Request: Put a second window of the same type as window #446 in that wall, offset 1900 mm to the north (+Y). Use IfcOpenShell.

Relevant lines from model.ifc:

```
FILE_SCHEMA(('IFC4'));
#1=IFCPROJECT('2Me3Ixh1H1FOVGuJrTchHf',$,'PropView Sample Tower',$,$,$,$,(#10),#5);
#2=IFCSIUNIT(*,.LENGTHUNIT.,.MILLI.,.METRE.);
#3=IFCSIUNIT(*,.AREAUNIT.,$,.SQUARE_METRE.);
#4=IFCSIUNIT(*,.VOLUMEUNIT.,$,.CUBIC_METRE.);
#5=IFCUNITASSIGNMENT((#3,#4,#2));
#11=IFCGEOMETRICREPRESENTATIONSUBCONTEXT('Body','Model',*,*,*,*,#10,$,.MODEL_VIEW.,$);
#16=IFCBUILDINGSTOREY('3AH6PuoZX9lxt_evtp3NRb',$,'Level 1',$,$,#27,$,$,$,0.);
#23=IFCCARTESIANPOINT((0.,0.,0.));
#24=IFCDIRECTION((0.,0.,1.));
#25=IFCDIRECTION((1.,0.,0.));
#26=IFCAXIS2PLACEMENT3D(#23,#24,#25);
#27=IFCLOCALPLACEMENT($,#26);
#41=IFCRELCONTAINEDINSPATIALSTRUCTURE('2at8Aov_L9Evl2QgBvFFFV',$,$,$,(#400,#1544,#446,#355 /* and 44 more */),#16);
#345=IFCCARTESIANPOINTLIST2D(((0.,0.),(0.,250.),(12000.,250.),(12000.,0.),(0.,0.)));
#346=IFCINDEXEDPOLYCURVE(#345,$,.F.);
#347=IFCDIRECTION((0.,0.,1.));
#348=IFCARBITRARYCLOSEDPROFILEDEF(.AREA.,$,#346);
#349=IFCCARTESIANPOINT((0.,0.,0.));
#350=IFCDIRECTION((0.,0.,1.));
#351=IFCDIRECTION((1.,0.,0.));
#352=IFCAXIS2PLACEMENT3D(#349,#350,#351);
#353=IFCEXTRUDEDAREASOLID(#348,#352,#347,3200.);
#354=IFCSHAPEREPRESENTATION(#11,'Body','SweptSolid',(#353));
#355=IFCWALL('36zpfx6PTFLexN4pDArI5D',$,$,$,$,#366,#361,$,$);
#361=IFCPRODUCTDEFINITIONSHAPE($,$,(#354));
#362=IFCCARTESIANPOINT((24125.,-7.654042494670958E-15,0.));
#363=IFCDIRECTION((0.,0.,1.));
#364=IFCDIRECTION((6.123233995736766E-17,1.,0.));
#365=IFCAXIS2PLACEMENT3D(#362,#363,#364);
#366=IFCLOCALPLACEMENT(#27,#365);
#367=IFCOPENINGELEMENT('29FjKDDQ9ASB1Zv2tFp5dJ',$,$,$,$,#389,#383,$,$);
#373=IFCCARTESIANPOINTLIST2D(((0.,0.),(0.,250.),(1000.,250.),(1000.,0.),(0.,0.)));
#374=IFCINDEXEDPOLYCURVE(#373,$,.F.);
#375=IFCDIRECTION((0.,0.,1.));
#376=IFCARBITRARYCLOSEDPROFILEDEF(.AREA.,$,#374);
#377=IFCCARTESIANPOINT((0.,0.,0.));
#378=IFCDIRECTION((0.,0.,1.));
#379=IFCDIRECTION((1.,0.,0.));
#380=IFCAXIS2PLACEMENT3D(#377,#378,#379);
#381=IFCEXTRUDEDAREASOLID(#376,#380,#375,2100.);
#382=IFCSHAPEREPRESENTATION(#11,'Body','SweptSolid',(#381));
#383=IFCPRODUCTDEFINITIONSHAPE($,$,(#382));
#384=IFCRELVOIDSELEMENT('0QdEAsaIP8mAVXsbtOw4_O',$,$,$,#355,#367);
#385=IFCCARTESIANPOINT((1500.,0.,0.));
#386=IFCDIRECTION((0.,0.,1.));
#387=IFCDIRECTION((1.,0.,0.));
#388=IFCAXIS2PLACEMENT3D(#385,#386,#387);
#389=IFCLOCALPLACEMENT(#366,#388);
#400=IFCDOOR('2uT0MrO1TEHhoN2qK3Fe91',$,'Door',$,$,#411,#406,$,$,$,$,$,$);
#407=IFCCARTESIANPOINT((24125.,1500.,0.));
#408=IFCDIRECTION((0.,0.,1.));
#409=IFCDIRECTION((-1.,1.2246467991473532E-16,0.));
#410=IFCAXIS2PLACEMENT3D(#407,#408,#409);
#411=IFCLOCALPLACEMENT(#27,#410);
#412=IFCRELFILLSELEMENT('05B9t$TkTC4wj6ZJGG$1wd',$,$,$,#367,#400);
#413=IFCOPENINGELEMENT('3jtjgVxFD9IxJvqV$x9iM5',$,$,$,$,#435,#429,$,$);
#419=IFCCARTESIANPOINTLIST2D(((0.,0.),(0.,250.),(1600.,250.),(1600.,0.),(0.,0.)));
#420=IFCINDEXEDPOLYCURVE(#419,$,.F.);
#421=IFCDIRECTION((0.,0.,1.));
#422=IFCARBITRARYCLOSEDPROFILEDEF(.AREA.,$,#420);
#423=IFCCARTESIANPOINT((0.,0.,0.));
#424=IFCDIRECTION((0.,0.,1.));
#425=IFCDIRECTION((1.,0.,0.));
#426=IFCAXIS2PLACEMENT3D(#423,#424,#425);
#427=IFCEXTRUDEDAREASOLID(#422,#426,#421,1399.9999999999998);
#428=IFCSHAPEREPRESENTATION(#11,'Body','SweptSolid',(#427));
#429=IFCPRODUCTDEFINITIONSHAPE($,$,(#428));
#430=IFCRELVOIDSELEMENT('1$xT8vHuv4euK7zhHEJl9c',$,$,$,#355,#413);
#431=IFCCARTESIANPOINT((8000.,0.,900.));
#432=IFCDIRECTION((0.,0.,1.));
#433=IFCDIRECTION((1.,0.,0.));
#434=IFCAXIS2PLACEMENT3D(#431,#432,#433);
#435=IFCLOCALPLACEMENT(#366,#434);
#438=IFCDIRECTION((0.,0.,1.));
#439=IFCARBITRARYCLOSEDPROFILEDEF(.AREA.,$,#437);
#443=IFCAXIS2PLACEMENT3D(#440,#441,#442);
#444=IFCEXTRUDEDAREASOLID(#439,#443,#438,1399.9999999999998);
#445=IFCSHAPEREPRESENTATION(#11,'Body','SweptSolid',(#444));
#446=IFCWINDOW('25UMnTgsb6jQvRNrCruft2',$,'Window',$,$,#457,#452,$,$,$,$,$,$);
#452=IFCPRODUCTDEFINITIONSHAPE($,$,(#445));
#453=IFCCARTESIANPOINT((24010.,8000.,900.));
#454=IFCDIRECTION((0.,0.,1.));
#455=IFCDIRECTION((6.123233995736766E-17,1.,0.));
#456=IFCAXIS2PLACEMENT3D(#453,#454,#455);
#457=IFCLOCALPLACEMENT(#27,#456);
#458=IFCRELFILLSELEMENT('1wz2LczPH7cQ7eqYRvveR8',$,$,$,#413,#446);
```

```python
import ifcopenshell
import ifcopenshell.api.feature
import ifcopenshell.api.geometry
import ifcopenshell.api.root
import ifcopenshell.geom
import ifcopenshell.util.element
import ifcopenshell.util.placement
import ifcopenshell.util.shape
import ifcopenshell.util.unit

model = ifcopenshell.open("model.ifc")
unit_scale = ifcopenshell.util.unit.calculate_unit_scale(model)
settings = ifcopenshell.geom.settings()


def volume(element):
    """Net volume in cubic metres, openings subtracted."""
    shape = ifcopenshell.geom.create_shape(settings, element)
    return ifcopenshell.util.shape.get_volume(shape.geometry)


window = model.by_guid("25UMnTgsb6jQvRNrCruft2")
opening = window.FillsVoids[0].RelatingOpeningElement
wall = opening.VoidsElements[0].RelatingBuildingElement
before = volume(wall)
shift = ifcopenshell.util.placement.get_local_placement(wall.ObjectPlacement)[:3, 0] * 1.9 / unit_scale

# copy_class copies the void relationship, type, container and properties, but no geometry.
new_opening = ifcopenshell.api.root.copy_class(model, product=opening)
new_opening.Representation = ifcopenshell.util.element.copy_deep(
    model, opening.Representation, exclude=["IfcGeometricRepresentationContext", "IfcRepresentationMap"]
)
new_window = ifcopenshell.api.root.copy_class(model, product=window)
new_window.Representation = ifcopenshell.util.element.copy_deep(
    model, window.Representation, exclude=["IfcGeometricRepresentationContext", "IfcRepresentationMap"]
)
ifcopenshell.api.feature.add_filling(model, opening=new_opening, element=new_window)

for old, new in ((opening, new_opening), (window, new_window)):
    matrix = ifcopenshell.util.placement.get_local_placement(old.ObjectPlacement)
    matrix[:3, 3] += shift
    ifcopenshell.api.geometry.edit_object_placement(model, product=new, matrix=matrix, is_si=False)

after = volume(wall)

print(f"wall volume {before:.3f} -> {after:.3f} m3")

model.write("model-out.ifc")
```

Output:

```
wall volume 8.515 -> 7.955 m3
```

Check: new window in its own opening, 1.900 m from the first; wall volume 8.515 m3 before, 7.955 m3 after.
